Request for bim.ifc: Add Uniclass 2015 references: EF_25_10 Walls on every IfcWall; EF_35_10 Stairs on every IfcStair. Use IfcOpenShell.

First a look at what the model holds.

```python
import ifcopenshell

model = ifcopenshell.open("bim.ifc")
print(model.schema)
print("classifications:", [c.Name for c in model.by_type("IfcClassification")])
for ifc_class in ("IfcDoor", "IfcRoof", "IfcStair", "IfcWall", "IfcWindow"):
    print(ifc_class, len(model.by_type(ifc_class)))
```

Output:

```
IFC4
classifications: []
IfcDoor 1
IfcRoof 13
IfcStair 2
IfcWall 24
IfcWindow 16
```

```python
import ifcopenshell
import ifcopenshell.api.classification

model = ifcopenshell.open("bim.ifc")

system = ifcopenshell.api.classification.add_classification(model, classification="Uniclass 2015")

codes = {
    "IfcWall": ("EF_25_10", "Walls"),
    "IfcStair": ("EF_35_10", "Stairs"),
}
for ifc_class, (code, name) in codes.items():
    products = model.by_type(ifc_class)
    ifcopenshell.api.classification.add_reference(
        model, products=products, classification=system, identification=code, name=name
    )
    print(code, len(products))

model.write("bim-out.ifc")
```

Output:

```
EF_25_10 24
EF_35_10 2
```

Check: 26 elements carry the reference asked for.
